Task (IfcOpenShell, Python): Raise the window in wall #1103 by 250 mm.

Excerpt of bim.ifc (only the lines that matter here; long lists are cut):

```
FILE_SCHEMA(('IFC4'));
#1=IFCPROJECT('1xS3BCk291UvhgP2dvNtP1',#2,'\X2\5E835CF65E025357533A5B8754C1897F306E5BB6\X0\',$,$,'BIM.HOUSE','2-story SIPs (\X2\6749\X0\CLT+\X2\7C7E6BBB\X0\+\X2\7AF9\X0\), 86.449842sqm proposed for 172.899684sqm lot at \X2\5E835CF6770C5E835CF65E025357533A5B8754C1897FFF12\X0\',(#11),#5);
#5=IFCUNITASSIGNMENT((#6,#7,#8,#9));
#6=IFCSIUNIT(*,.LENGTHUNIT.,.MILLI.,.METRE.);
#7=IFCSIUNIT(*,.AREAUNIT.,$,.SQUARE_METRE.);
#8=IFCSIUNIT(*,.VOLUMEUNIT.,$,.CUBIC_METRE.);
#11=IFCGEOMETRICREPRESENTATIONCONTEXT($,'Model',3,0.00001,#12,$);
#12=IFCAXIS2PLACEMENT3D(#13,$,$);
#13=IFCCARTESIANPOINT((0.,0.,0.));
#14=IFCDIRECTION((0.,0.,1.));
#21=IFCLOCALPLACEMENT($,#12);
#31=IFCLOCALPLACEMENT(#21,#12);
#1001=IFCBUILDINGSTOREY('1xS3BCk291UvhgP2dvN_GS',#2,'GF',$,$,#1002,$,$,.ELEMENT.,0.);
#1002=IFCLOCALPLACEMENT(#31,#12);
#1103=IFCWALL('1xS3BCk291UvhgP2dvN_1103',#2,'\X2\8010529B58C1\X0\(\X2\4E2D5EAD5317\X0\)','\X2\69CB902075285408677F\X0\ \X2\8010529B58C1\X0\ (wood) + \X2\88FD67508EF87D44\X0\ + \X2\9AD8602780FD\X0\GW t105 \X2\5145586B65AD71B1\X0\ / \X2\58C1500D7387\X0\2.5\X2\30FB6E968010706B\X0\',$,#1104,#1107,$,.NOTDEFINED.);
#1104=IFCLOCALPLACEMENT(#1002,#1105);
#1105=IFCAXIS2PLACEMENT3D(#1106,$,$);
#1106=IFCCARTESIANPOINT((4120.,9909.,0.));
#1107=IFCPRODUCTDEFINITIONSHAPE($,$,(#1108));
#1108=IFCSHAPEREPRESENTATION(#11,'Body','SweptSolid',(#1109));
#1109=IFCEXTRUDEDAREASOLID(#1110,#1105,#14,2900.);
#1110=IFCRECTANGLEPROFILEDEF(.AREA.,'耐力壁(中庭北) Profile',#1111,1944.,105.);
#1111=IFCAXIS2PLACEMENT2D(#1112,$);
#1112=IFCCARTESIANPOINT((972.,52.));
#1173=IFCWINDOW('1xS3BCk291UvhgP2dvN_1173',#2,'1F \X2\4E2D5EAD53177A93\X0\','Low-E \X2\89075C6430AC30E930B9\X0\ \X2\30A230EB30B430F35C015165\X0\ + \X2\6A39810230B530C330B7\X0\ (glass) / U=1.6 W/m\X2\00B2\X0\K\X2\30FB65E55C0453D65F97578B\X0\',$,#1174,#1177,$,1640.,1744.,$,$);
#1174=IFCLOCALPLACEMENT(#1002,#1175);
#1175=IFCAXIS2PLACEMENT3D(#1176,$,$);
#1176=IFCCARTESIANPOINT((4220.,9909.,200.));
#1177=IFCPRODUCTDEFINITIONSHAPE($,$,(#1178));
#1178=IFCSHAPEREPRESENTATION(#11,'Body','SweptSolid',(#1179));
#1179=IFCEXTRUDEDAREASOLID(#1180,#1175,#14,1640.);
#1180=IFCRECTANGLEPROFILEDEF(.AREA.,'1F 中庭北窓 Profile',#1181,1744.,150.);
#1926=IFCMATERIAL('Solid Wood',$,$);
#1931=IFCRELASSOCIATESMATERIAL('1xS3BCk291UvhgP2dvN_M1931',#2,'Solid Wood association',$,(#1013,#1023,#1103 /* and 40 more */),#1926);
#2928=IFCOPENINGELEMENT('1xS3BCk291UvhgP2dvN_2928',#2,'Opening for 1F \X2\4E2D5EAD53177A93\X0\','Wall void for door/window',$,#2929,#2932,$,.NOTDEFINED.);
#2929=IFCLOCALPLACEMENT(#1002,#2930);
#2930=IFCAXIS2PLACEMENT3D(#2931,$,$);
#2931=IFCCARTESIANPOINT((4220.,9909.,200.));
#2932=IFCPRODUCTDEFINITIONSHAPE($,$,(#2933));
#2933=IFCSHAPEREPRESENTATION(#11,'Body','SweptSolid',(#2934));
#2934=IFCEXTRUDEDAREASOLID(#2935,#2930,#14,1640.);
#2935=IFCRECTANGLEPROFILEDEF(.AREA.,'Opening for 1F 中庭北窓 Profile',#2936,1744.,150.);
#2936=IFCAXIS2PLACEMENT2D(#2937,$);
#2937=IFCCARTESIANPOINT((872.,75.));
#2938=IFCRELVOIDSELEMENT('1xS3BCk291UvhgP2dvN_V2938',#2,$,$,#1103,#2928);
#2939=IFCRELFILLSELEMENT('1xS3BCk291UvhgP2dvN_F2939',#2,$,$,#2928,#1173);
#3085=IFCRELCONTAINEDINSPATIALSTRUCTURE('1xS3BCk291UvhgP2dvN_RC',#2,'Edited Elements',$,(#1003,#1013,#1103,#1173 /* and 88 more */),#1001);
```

```python
import numpy as np
import ifcopenshell
import ifcopenshell.api.geometry
import ifcopenshell.util.placement
import ifcopenshell.util.unit

model = ifcopenshell.open("bim.ifc")
unit_scale = ifcopenshell.util.unit.calculate_unit_scale(model)

window = model.by_guid("1xS3BCk291UvhgP2dvN_1173")
opening = window.FillsVoids[0].RelatingOpeningElement
dz = 0.25 / unit_scale

shift = np.array([0.0, 0.0, dz])
# The window is not placed relative to its opening, so move both.
for product in (opening, window):
    matrix = ifcopenshell.util.placement.get_local_placement(product.ObjectPlacement)
    matrix[:3, 3] += shift
    ifcopenshell.api.geometry.edit_object_placement(model, product=product, matrix=matrix, is_si=False)

print(f"moved by {dz * unit_scale:+.3f} m")

model.write("bim_updated.ifc")
```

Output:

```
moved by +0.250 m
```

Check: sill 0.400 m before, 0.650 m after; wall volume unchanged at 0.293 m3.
